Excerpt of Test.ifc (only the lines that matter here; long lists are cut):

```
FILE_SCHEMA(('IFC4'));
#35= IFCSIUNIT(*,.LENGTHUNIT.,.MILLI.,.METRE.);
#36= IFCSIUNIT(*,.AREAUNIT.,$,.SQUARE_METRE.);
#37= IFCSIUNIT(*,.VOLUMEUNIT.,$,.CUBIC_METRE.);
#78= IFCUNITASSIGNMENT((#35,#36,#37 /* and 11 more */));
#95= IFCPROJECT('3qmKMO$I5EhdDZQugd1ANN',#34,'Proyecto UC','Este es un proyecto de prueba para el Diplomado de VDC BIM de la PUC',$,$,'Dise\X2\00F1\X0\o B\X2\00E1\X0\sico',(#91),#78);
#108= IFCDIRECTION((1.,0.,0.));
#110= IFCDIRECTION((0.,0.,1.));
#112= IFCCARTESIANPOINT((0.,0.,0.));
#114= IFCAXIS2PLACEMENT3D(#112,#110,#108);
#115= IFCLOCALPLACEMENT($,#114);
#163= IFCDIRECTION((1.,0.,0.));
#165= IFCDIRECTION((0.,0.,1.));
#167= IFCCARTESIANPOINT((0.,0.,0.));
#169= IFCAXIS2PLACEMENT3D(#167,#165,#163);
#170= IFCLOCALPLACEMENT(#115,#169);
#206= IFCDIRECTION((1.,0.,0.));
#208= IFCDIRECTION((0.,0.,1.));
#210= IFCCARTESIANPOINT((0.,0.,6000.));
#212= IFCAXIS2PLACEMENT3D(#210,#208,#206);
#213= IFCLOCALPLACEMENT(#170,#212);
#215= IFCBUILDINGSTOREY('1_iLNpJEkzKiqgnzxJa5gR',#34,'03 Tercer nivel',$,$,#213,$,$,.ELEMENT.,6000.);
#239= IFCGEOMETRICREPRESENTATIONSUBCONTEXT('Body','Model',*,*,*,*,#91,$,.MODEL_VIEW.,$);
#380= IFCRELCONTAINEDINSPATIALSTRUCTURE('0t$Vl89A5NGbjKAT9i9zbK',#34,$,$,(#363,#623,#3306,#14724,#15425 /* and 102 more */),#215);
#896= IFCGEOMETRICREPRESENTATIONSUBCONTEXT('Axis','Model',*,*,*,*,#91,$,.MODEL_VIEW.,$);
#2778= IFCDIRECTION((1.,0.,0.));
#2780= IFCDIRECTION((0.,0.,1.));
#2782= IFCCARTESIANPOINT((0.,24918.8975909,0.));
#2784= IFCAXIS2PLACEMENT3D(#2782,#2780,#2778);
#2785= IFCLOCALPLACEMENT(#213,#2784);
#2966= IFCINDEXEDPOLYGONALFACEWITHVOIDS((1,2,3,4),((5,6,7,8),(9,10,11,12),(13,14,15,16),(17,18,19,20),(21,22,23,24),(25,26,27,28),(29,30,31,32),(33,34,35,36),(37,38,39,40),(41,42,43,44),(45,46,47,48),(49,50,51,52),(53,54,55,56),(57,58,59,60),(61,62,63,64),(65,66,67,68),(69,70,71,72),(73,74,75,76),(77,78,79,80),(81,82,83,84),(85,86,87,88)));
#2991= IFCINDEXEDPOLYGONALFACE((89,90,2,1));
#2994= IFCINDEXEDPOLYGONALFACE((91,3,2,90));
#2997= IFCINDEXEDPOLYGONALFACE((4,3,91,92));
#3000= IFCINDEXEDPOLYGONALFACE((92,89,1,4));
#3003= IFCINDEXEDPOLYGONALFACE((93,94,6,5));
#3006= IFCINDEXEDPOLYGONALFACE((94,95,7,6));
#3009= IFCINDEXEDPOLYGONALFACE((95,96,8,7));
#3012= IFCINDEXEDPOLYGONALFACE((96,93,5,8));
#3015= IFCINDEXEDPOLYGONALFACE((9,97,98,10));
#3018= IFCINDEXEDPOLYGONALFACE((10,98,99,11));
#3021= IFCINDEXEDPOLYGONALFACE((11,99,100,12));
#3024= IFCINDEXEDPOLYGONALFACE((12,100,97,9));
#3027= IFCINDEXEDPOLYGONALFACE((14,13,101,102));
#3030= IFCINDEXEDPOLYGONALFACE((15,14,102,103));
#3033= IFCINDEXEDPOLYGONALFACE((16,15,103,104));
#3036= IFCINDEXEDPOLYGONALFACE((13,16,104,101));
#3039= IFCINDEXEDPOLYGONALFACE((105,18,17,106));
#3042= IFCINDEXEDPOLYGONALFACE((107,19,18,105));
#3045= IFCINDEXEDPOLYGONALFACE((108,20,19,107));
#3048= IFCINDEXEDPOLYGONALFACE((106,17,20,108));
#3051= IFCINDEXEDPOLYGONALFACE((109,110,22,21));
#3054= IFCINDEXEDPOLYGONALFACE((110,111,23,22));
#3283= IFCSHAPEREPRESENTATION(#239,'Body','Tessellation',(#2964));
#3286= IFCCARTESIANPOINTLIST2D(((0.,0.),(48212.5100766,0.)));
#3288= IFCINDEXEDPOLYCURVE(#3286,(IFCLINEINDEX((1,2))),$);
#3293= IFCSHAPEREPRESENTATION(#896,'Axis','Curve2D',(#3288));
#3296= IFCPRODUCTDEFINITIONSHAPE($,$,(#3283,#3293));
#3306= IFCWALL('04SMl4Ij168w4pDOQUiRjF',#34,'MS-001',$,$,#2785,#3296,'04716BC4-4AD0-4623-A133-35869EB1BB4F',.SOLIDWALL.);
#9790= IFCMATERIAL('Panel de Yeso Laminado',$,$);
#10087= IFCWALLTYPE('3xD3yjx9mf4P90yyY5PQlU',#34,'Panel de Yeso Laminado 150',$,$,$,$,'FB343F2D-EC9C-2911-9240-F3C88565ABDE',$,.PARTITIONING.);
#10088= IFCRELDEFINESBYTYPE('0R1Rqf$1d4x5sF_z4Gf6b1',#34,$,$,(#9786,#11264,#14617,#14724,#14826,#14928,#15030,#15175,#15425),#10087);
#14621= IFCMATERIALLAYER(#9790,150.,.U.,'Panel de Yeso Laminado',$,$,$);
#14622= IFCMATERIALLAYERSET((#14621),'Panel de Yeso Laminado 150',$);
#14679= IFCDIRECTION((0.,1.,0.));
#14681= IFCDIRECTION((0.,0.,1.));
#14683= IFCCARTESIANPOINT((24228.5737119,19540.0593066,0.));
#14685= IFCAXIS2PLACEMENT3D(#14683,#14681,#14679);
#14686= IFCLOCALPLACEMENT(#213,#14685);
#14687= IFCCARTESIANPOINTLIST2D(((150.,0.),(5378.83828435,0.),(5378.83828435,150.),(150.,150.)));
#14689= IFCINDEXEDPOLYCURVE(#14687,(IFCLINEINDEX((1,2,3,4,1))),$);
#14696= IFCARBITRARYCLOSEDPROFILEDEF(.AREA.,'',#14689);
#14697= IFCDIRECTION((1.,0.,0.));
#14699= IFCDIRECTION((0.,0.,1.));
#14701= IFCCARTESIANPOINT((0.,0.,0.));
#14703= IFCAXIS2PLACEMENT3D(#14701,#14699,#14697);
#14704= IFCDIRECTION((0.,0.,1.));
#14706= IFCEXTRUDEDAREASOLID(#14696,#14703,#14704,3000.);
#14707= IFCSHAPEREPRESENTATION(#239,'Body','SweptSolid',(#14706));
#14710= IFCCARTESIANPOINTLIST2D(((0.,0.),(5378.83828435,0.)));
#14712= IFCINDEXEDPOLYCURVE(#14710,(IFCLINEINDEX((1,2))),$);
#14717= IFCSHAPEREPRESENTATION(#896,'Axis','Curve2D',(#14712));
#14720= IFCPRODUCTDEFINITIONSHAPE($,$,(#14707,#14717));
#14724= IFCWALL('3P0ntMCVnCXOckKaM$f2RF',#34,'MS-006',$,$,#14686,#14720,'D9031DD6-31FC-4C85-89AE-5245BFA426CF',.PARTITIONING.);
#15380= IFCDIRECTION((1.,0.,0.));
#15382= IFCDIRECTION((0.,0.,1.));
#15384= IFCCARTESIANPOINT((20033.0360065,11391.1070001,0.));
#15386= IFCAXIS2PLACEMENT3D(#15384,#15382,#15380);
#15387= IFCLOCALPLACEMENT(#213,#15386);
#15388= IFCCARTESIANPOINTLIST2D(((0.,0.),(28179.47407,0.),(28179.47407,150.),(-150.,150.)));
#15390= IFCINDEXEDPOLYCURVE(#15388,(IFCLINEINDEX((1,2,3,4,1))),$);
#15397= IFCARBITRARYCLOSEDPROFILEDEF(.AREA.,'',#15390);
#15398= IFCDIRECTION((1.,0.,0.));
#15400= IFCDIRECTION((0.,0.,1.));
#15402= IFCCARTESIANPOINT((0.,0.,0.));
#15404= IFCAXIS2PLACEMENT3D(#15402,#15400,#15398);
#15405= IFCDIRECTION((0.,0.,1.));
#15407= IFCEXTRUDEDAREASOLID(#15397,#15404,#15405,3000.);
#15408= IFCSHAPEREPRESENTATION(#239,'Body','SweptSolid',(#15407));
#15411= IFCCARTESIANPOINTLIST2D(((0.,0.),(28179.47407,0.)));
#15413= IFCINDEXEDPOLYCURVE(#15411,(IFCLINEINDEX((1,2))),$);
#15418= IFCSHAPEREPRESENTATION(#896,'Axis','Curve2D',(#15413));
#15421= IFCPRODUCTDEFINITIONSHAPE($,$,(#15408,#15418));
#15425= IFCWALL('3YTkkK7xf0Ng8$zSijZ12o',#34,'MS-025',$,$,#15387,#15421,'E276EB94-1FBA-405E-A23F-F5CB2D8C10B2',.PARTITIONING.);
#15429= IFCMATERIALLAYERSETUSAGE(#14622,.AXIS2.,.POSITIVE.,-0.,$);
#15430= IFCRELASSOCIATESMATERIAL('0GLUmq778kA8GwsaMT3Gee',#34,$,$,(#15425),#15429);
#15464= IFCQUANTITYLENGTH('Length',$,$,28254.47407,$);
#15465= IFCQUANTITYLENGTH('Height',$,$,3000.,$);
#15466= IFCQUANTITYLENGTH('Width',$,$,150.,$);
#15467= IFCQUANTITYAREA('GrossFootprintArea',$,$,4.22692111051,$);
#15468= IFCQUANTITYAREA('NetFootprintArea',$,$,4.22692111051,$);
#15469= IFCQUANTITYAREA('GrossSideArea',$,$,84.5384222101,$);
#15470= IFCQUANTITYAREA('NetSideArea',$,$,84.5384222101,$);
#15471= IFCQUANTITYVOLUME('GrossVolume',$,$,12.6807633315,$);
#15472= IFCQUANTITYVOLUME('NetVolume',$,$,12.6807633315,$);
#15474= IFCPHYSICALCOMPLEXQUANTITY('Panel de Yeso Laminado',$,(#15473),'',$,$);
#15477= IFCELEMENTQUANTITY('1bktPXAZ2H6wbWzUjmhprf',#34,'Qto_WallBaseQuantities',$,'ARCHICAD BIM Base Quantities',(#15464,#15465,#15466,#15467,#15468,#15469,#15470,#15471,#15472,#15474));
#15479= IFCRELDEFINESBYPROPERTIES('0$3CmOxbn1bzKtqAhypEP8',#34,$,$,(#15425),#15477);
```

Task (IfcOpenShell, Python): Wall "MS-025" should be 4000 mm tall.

```python
import ifcopenshell
import ifcopenshell.api.pset
import ifcopenshell.geom
import ifcopenshell.util.element
import ifcopenshell.util.representation
import ifcopenshell.util.shape
import ifcopenshell.util.unit

model = ifcopenshell.open("Test.ifc")
unit_scale = ifcopenshell.util.unit.calculate_unit_scale(model)
area_scale = ifcopenshell.util.unit.calculate_unit_scale(model, "AREAUNIT")
volume_scale = ifcopenshell.util.unit.calculate_unit_scale(model, "VOLUMEUNIT")
settings = ifcopenshell.geom.settings()


def volume(element):
    """Net volume in cubic metres, openings subtracted."""
    shape = ifcopenshell.geom.create_shape(settings, element)
    return ifcopenshell.util.shape.get_volume(shape.geometry)


wall = model.by_guid("3YTkkK7xf0Ng8$zSijZ12o")
before = volume(wall)

body = ifcopenshell.util.representation.get_representation(wall, "Model", "Body")
solid = body.Items[0]
old_height = solid.Depth
solid.Depth = 4 / unit_scale
after = volume(wall)
thickness = 0.15  # wall thickness in metres

# Update the stored height, areas and volumes.
qto = model.by_id(ifcopenshell.util.element.get_pset(wall, "Qto_WallBaseQuantities", should_inherit=False)["id"])
ifcopenshell.api.pset.edit_qto(model, qto=qto, properties={
    "Height": solid.Depth,
    "GrossSideArea": ifcopenshell.util.element.get_pset(wall, "Qto_WallBaseQuantities", "GrossSideArea") * solid.Depth / old_height,
    "NetSideArea": after / thickness / area_scale,
    "GrossVolume": ifcopenshell.util.element.get_pset(wall, "Qto_WallBaseQuantities", "GrossVolume") * solid.Depth / old_height,
    "NetVolume": after / volume_scale,
})

print(f"height {old_height:g} -> {solid.Depth:g}, volume {before:.3f} -> {after:.3f} m3")

model.write("Test_edited.ifc")
```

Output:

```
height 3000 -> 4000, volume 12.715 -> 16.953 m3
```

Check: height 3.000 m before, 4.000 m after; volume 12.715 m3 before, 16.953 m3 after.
